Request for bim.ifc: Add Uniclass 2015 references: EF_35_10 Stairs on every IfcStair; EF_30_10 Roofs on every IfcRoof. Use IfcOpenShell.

First a look at what the model holds.

```python
import ifcopenshell

model = ifcopenshell.open("bim.ifc")
print(model.schema)
print("classifications:", [c.Name for c in model.by_type("IfcClassification")])
for ifc_class in ("IfcDoor", "IfcRoof", "IfcStair", "IfcWall", "IfcWindow"):
    print(ifc_class, len(model.by_type(ifc_class)))
```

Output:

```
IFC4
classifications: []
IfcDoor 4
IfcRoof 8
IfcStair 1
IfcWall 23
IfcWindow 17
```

```python
import ifcopenshell
import ifcopenshell.api.classification

model = ifcopenshell.open("bim.ifc")

system = ifcopenshell.api.classification.add_classification(model, classification="Uniclass 2015")

codes = {
    "IfcStair": ("EF_35_10", "Stairs"),
    "IfcRoof": ("EF_30_10", "Roofs"),
}
for ifc_class, (code, name) in codes.items():
    products = model.by_type(ifc_class)
    ifcopenshell.api.classification.add_reference(
        model, products=products, classification=system, identification=code, name=name
    )
    print(code, len(products))

model.write("bim-out.ifc")
```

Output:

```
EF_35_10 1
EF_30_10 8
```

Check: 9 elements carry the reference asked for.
